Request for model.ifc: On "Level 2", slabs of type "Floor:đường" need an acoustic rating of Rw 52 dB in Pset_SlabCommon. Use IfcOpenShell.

First a look at what the model holds.

```python
import ifcopenshell
import ifcopenshell.util.element

model = ifcopenshell.open("model.ifc")
print(model.schema)
storey = next(s for s in model.by_type("IfcBuildingStorey") if s.Name == "Level 2")
slabs = [e for e in ifcopenshell.util.element.get_decomposition(storey) if e.is_a("IfcSlab")]
seen = {}
for e in slabs:
    element_type = ifcopenshell.util.element.get_type(e)
    key = (element_type.Name if element_type != e and element_type else None, ifcopenshell.util.element.get_pset(e, "Pset_SlabCommon", "AcousticRating"))
    seen[key] = seen.get(key, 0) + 1
for (name, value), count in sorted(seen.items(), key=str):
    print(count, "x", name, "|", value)
```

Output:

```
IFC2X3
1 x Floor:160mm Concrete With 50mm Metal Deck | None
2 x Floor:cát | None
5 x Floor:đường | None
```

```python
import ifcopenshell
import ifcopenshell.api.pset
import ifcopenshell.util.element

model = ifcopenshell.open("model.ifc")

storey = next(s for s in model.by_type("IfcBuildingStorey") if s.Name == "Level 2")
slabs = [e for e in ifcopenshell.util.element.get_decomposition(storey) if e.is_a("IfcSlab")]

count = 0
for e in slabs:
    element_type = ifcopenshell.util.element.get_type(e)
    if element_type in (None, e) or element_type.Name != "Floor:đường":
        continue
    # add_pset returns the element's existing set when there is one.
    pset = ifcopenshell.api.pset.add_pset(model, product=e, name="Pset_SlabCommon")
    ifcopenshell.api.pset.edit_pset(model, pset=pset, properties={"AcousticRating": "Rw 52 dB"})
    count += 1

print(count, "slabs updated")

model.write("model-out.ifc")
```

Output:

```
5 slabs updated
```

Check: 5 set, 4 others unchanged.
